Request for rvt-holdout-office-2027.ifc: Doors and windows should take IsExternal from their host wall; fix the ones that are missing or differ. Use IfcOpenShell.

First a look at what the model holds.

```python
import ifcopenshell
import ifcopenshell.util.element

model = ifcopenshell.open("rvt-holdout-office-2027.ifc")
print(model.schema)
seen = {}
for e in model.by_type("IfcDoor") + model.by_type("IfcWindow"):
    if not e.FillsVoids:
        continue
    host = e.FillsVoids[0].RelatingOpeningElement.VoidsElements[0].RelatingBuildingElement
    own = ifcopenshell.util.element.get_pset(e, f"Pset_{e.is_a()[3:].removesuffix('StandardCase')}Common", "IsExternal")
    wall = ifcopenshell.util.element.get_pset(host, "Pset_WallCommon", "IsExternal")
    seen[e.is_a(), own, wall] = seen.get((e.is_a(), own, wall), 0) + 1
for (cls, own, wall), count in sorted(seen.items(), key=str):
    print(count, cls, "IsExternal:", own, "| host wall:", wall)
```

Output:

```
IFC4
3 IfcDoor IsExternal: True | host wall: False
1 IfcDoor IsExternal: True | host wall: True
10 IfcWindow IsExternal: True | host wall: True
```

```python
import ifcopenshell
import ifcopenshell.api.pset
import ifcopenshell.util.element

model = ifcopenshell.open("rvt-holdout-office-2027.ifc")

count = 0
for ifc_class, pset_name in (("IfcDoor", "Pset_DoorCommon"), ("IfcWindow", "Pset_WindowCommon")):
    for e in model.by_type(ifc_class):
        if not e.FillsVoids:
            continue
        host = e.FillsVoids[0].RelatingOpeningElement.VoidsElements[0].RelatingBuildingElement
        external = ifcopenshell.util.element.get_pset(host, "Pset_WallCommon", "IsExternal")
        if external is None or ifcopenshell.util.element.get_pset(e, pset_name, "IsExternal") == external:
            continue
        pset = ifcopenshell.api.pset.add_pset(model, product=e, name=pset_name)
        ifcopenshell.api.pset.edit_pset(model, pset=pset, properties={"IsExternal": external})
        count += 1

print(count, "updated")

model.write("rvt-holdout-office-2027_edited.ifc")
```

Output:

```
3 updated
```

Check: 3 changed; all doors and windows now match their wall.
